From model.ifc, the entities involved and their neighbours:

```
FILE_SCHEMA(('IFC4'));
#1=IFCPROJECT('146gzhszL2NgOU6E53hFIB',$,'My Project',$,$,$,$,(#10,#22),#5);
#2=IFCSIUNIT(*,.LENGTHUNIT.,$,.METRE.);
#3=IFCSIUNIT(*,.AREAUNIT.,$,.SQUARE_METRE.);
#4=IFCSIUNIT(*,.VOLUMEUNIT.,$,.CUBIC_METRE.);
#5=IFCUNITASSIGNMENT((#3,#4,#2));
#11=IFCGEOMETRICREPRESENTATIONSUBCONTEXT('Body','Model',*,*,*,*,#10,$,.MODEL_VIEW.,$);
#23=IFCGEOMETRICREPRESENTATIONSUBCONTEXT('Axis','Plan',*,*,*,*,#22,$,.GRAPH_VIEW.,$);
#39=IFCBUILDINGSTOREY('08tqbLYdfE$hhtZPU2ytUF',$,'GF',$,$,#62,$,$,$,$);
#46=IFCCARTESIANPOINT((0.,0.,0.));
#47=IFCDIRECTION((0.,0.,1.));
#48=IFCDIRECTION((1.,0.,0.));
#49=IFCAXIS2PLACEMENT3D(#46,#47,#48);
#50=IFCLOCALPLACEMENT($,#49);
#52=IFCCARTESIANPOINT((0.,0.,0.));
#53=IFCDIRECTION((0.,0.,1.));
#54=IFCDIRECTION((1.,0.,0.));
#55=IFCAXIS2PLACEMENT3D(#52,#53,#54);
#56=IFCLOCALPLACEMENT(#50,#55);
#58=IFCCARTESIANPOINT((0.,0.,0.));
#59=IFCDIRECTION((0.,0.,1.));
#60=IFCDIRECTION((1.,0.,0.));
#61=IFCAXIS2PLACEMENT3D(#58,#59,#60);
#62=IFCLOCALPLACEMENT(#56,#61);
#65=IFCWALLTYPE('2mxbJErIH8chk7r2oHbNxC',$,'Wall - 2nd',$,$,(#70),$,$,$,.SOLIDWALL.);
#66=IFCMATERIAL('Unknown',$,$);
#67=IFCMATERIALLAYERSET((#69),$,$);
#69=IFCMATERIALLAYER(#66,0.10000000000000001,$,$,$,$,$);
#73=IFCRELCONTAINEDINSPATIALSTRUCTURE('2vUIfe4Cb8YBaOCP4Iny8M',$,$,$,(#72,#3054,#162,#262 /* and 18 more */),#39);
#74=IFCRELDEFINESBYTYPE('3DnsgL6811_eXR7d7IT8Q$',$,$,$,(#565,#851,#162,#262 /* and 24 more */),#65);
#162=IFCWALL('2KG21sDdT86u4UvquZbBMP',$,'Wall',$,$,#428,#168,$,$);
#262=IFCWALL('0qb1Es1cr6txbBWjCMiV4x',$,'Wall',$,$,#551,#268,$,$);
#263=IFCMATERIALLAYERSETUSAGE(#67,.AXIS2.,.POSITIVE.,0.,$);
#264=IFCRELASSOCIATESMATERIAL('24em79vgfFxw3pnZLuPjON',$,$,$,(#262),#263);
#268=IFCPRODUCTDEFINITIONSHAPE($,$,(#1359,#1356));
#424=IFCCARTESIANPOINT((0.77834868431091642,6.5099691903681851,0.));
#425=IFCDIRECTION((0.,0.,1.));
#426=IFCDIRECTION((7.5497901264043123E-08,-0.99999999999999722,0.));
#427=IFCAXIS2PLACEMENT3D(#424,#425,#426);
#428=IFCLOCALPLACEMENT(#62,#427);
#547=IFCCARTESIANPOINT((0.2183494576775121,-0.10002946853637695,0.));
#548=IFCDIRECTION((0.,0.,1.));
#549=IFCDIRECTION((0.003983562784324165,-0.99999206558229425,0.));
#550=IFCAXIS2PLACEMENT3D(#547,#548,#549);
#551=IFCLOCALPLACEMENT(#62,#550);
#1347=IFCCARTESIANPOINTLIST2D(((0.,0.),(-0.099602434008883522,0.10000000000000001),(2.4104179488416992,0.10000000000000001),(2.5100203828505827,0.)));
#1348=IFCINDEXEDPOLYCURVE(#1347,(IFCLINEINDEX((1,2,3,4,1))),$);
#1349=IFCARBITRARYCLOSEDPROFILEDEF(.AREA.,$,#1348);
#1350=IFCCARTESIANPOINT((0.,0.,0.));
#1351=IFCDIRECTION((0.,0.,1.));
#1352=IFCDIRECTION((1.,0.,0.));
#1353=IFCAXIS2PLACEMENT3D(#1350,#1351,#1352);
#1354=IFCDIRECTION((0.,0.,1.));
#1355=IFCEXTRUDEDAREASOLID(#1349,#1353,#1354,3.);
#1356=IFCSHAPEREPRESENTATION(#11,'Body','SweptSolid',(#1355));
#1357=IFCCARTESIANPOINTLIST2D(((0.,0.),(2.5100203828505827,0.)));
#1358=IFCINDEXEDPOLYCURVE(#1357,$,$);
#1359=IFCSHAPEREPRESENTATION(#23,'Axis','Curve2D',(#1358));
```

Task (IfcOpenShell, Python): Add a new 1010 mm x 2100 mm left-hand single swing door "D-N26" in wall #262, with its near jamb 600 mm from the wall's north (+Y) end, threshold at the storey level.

```python
import numpy as np
import ifcopenshell
import ifcopenshell.api.feature
import ifcopenshell.api.geometry
import ifcopenshell.api.root
import ifcopenshell.api.spatial
import ifcopenshell.geom
import ifcopenshell.util.element
import ifcopenshell.util.placement
import ifcopenshell.util.representation
import ifcopenshell.util.shape
import ifcopenshell.util.unit

model = ifcopenshell.open("model.ifc")
unit_scale = ifcopenshell.util.unit.calculate_unit_scale(model)
settings = ifcopenshell.geom.settings()


def volume(element):
    """Net volume in cubic metres, openings subtracted."""
    shape = ifcopenshell.geom.create_shape(settings, element)
    return ifcopenshell.util.shape.get_volume(shape.geometry)


wall = model.by_id(262)
storey = ifcopenshell.util.element.get_container(wall, ifc_class="IfcBuildingStorey")
context = ifcopenshell.util.representation.get_context(model, "Model", "Body", "MODEL_VIEW")
before = volume(wall)

width, height, from_end, sill = 1.01, 2.1, 0.6, 0.0  # metres

# The wall runs along its own X axis, and the end named is its -X end.
wall_shape = ifcopenshell.geom.create_shape(settings, wall)
x, y, z = ifcopenshell.util.shape.get_vertices(wall_shape.geometry).T
start = x.min() + from_end
face, thickness = float(y.min()), float(y.max() - y.min())
wall_matrix = ifcopenshell.util.placement.get_local_placement(wall.ObjectPlacement)
level = ifcopenshell.util.placement.get_local_placement(storey.ObjectPlacement)[2, 3]


def in_wall(x, y):
    """Placement at x, y metres in the wall's axes, at sill height."""
    matrix = wall_matrix.copy()
    matrix[:, 3] = wall_matrix @ np.array([x / unit_scale, y / unit_scale, 0.0, 1.0])
    matrix[2, 3] = level + sill / unit_scale
    return matrix


# Opening: a box that overshoots both wall faces by 50 mm.
opening = ifcopenshell.api.root.create_entity(model, ifc_class="IfcOpeningElement", predefined_type="OPENING")
box = ifcopenshell.api.geometry.add_wall_representation(
    model, context=context, length=width, height=height, thickness=thickness + 0.1
)
ifcopenshell.api.geometry.assign_representation(model, product=opening, representation=box)
ifcopenshell.api.geometry.edit_object_placement(model, product=opening, matrix=in_wall(start, face - 0.05), is_si=False)
ifcopenshell.api.feature.add_feature(model, feature=opening, element=wall)

door = ifcopenshell.api.root.create_entity(model, ifc_class="IfcDoor", name="D-N26", predefined_type="DOOR")
door.OverallWidth, door.OverallHeight = width / unit_scale, height / unit_scale
door.OperationType = "SINGLE_SWING_LEFT"
body = ifcopenshell.api.geometry.add_door_representation(
    model,
    context=context,
    overall_width=door.OverallWidth,
    overall_height=door.OverallHeight,
    operation_type="SINGLE_SWING_LEFT",
    lining_properties={"LiningDepth": thickness / unit_scale, "ThresholdDepth": thickness / unit_scale},
)
ifcopenshell.api.geometry.assign_representation(model, product=door, representation=body)
ifcopenshell.api.spatial.assign_container(model, products=[door], relating_structure=storey)
ifcopenshell.api.feature.add_filling(model, opening=opening, element=door)

# The lining spans the wall, so the door starts at the wall face.
ifcopenshell.api.geometry.edit_object_placement(model, product=door, matrix=in_wall(start, face), is_si=False)

after = volume(wall)

print(f"wall volume {before:.3f} -> {after:.3f} m3")

model.write("model_edited.ifc")
```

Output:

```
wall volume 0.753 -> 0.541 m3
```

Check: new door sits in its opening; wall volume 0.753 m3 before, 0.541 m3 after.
